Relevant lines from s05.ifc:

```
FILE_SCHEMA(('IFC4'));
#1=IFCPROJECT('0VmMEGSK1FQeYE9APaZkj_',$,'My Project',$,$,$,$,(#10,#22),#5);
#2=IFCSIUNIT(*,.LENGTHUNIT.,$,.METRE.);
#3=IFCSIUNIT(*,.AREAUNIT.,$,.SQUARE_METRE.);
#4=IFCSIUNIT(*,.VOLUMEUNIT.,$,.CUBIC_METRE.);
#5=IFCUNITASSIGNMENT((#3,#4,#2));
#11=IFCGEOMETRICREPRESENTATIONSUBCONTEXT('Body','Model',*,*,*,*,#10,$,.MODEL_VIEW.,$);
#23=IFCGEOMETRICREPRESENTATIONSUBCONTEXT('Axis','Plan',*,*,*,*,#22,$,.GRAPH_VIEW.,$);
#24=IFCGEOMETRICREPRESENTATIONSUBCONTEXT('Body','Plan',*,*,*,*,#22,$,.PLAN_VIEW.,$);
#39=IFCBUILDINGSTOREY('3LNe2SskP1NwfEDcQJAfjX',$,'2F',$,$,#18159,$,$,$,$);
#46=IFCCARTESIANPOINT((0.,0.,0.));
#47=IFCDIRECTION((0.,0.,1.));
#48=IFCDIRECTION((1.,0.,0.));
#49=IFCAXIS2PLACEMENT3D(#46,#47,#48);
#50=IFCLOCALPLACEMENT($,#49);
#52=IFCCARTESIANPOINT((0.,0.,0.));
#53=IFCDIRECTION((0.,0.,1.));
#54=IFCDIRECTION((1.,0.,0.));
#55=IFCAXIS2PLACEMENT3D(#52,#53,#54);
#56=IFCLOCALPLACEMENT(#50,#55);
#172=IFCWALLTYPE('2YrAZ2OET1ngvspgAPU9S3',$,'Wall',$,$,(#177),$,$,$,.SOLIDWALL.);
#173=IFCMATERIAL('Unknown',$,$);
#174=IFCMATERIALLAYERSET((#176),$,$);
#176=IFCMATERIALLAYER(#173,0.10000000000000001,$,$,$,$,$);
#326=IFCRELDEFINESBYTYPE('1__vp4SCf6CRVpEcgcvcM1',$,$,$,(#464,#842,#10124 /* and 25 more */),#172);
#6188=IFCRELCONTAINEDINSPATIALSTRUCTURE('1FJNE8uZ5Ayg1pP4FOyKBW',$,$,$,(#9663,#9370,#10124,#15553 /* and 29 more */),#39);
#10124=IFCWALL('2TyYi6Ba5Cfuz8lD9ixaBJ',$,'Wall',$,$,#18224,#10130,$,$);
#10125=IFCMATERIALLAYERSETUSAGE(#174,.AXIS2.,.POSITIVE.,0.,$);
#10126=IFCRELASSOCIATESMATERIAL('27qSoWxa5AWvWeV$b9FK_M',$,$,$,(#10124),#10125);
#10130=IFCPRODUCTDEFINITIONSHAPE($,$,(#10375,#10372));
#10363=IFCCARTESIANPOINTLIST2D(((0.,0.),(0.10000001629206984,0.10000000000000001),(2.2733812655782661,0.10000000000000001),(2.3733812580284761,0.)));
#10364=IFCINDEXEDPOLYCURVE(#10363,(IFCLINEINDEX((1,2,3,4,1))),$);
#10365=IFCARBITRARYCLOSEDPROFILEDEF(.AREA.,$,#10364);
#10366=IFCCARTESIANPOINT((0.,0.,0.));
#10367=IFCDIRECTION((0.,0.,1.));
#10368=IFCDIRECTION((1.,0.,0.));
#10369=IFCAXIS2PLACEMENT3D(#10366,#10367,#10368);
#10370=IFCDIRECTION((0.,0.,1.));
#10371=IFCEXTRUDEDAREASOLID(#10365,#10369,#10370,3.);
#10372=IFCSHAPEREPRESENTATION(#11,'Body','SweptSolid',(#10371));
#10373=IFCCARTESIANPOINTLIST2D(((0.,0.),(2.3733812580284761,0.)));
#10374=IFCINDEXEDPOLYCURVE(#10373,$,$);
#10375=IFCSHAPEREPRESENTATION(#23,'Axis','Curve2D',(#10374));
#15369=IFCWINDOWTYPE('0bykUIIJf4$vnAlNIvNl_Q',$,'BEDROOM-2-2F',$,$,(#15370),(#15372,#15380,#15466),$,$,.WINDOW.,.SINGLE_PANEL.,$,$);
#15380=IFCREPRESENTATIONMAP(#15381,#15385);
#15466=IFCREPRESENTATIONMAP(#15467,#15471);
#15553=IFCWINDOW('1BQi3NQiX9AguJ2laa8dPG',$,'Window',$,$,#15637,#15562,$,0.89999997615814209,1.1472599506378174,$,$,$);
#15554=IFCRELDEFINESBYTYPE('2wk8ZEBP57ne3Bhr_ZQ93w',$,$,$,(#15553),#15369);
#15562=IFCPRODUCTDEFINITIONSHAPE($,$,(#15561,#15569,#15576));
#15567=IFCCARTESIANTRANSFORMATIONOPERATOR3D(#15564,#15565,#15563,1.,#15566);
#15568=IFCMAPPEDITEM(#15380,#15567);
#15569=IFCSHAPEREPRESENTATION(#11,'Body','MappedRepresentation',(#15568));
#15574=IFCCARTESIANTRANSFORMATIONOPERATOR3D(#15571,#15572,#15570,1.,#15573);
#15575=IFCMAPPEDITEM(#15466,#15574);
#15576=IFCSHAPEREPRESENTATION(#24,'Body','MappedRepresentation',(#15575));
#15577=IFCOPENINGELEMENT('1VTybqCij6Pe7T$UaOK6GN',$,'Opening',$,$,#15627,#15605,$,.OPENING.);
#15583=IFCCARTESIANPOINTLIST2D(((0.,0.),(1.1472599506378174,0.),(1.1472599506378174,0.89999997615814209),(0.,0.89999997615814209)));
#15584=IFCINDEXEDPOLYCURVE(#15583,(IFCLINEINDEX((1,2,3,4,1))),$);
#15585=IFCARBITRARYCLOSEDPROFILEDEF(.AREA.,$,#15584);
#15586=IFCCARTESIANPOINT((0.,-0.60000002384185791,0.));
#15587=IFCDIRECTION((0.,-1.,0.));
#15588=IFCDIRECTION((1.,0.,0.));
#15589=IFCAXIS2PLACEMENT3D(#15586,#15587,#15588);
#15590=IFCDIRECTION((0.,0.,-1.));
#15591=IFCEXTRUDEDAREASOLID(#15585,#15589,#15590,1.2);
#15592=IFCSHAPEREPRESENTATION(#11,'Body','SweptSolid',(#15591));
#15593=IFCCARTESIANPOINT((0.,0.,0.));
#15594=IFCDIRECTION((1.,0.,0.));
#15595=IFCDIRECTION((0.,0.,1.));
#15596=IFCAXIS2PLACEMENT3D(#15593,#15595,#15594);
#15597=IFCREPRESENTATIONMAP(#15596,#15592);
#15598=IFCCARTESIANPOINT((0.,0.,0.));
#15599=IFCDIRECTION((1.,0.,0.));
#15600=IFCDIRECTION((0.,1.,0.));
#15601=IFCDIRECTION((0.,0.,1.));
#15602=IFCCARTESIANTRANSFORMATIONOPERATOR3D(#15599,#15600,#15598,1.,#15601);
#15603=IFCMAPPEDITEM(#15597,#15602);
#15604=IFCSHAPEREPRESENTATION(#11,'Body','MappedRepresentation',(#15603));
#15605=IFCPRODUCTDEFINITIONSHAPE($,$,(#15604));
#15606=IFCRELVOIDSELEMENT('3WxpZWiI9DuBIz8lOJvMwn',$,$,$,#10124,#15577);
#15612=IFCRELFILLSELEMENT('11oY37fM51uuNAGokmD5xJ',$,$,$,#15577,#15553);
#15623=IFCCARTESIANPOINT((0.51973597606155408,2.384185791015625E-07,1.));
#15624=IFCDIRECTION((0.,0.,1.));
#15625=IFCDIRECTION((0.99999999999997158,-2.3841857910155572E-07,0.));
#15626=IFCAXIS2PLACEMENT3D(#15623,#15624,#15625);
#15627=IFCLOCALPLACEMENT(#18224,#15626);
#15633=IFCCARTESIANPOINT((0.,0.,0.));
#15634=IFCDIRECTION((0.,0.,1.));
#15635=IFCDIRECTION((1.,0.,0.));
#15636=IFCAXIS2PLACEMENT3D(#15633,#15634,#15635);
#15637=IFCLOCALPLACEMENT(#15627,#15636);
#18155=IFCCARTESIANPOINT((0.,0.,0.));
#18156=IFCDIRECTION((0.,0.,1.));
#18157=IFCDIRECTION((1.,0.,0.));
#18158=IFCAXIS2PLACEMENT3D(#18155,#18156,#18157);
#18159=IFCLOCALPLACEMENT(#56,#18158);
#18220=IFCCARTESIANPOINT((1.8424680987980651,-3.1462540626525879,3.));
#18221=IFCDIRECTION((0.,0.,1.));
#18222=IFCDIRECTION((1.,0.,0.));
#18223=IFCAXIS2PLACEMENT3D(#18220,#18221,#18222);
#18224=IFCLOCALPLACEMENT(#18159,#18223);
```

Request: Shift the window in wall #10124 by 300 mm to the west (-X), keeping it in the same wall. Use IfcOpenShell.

```python
import ifcopenshell
import ifcopenshell.api.geometry
import ifcopenshell.util.placement
import ifcopenshell.util.unit

model = ifcopenshell.open("s05.ifc")
unit_scale = ifcopenshell.util.unit.calculate_unit_scale(model)

window = model.by_guid("1BQi3NQiX9AguJ2laa8dPG")
opening = window.FillsVoids[0].RelatingOpeningElement
wall = opening.VoidsElements[0].RelatingBuildingElement

wall_matrix = ifcopenshell.util.placement.get_local_placement(wall.ObjectPlacement)
shift = wall_matrix[:3, 0] * -0.3 / unit_scale
before = ifcopenshell.util.placement.get_local_placement(window.ObjectPlacement)[:3, 3].copy()

# The window is placed relative to its opening, so it follows when the opening moves.
matrix = ifcopenshell.util.placement.get_local_placement(opening.ObjectPlacement)
matrix[:3, 3] += shift
ifcopenshell.api.geometry.edit_object_placement(
    model, product=opening, matrix=matrix, is_si=False, should_transform_children=True
)

after = ifcopenshell.util.placement.get_local_placement(window.ObjectPlacement)[:3, 3]
print("window moved by", (after - before).round(3) + 0.0)

model.write("s05_rev.ifc")
```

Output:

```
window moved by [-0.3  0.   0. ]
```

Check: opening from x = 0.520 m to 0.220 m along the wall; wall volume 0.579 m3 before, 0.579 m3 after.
